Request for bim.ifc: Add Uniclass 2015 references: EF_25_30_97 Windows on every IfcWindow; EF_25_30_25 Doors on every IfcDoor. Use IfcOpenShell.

First a look at what the model holds.

```python
import ifcopenshell

model = ifcopenshell.open("bim.ifc")
print(model.schema)
print("classifications:", [c.Name for c in model.by_type("IfcClassification")])
for ifc_class in ("IfcDoor", "IfcRoof", "IfcStair", "IfcWall", "IfcWindow"):
    print(ifc_class, len(model.by_type(ifc_class)))
```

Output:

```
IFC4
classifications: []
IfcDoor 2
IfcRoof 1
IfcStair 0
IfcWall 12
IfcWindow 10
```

```python
import ifcopenshell
import ifcopenshell.api.classification

model = ifcopenshell.open("bim.ifc")

system = ifcopenshell.api.classification.add_classification(model, classification="Uniclass 2015")

codes = {
    "IfcWindow": ("EF_25_30_97", "Windows"),
    "IfcDoor": ("EF_25_30_25", "Doors"),
}
for ifc_class, (code, name) in codes.items():
    products = model.by_type(ifc_class)
    ifcopenshell.api.classification.add_reference(
        model, products=products, classification=system, identification=code, name=name
    )
    print(code, len(products))

model.write("bim_rev.ifc")
```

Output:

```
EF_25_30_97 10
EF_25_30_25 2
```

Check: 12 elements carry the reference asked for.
